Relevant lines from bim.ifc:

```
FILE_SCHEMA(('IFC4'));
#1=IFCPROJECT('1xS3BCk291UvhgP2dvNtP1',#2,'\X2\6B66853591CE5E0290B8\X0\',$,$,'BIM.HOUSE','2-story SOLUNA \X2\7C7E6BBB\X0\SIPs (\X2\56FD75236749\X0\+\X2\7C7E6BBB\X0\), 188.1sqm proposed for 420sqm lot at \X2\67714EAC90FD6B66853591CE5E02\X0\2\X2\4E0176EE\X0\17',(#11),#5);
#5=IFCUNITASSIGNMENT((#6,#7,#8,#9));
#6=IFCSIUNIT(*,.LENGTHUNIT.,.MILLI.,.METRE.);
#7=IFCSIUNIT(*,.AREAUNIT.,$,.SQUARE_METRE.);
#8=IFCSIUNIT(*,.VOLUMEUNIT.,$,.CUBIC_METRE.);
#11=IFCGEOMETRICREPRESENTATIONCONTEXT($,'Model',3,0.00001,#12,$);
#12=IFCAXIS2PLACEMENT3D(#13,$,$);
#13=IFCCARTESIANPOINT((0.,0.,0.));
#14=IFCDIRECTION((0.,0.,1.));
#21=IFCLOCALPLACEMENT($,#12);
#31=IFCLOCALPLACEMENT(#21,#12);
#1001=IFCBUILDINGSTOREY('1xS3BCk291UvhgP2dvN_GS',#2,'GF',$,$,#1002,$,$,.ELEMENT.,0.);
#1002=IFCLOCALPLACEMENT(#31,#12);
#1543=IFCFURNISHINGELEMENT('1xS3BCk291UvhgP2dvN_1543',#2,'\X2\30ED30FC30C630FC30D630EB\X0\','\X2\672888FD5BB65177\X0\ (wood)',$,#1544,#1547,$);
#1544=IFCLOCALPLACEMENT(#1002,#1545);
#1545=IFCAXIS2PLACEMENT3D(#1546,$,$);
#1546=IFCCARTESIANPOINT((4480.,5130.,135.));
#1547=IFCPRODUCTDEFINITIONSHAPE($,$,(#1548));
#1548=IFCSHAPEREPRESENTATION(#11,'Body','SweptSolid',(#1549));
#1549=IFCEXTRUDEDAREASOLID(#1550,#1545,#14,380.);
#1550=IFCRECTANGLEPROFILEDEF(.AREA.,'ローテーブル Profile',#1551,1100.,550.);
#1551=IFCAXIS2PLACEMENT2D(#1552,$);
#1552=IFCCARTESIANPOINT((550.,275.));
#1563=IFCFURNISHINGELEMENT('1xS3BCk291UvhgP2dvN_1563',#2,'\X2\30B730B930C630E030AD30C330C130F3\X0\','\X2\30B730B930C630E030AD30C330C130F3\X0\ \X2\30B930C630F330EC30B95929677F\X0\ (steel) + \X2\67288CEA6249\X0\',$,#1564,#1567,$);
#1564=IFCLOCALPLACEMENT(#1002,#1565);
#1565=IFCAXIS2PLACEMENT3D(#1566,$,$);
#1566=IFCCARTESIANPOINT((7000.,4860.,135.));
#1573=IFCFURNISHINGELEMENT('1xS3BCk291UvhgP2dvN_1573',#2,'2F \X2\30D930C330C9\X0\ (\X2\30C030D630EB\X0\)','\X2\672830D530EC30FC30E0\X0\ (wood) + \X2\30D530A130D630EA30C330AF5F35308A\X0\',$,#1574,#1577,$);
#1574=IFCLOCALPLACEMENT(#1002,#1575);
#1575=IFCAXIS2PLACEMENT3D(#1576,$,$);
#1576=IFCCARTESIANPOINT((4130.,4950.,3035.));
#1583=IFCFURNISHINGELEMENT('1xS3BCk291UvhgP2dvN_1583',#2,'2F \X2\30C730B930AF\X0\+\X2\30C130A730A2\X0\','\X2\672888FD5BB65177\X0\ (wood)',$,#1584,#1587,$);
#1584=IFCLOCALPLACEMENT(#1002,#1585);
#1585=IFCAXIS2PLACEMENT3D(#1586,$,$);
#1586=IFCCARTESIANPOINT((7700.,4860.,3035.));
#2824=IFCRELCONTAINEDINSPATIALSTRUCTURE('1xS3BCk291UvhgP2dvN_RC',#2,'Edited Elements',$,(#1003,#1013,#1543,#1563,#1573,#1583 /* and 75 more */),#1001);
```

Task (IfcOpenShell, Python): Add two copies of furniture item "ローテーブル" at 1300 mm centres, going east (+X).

```python
import numpy as np
import ifcopenshell
import ifcopenshell.api.geometry
import ifcopenshell.api.root
import ifcopenshell.util.element
import ifcopenshell.util.placement
import ifcopenshell.util.unit

model = ifcopenshell.open("bim.ifc")
unit_scale = ifcopenshell.util.unit.calculate_unit_scale(model)


def reuse_history(source, copy):
    """copy_class also copies each property set's owner history, people and application; keep the originals."""
    for rel in copy.IsDefinedBy:
        if rel.is_a("IfcRelDefinesByProperties") and (history := rel.RelatingPropertyDefinition.OwnerHistory):
            rel.RelatingPropertyDefinition.OwnerHistory = source.OwnerHistory
            ifcopenshell.util.element.remove_deep2(model, history)


source = model.by_guid("1xS3BCk291UvhgP2dvN_1543")
base = ifcopenshell.util.placement.get_local_placement(source.ObjectPlacement)
step = np.array([1.0, 0.0, 0.0]) * 1.3 / unit_scale

for i in range(1, 3):
    copy = ifcopenshell.api.root.copy_class(model, product=source)
    copy.Representation = ifcopenshell.util.element.copy_deep(
        model, source.Representation, exclude=["IfcGeometricRepresentationContext", "IfcRepresentationMap"]
    )
    reuse_history(source, copy)
    matrix = base.copy()
    matrix[:3, 3] += i * step
    print("added at", matrix[:3, 3].round(3) + 0.0)
    ifcopenshell.api.geometry.edit_object_placement(model, product=copy, matrix=matrix, is_si=False)

model.write("bim_rev.ifc")
```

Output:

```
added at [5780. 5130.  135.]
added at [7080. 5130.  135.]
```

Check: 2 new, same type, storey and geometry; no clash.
